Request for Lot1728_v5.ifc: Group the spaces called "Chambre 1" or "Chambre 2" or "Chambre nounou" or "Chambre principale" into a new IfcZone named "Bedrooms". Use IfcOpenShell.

First a look at what the model holds.

```python
import ifcopenshell

model = ifcopenshell.open("Lot1728_v5.ifc")
print(model.schema)
seen = {}
for space in model.by_type("IfcSpace"):
    seen[space.LongName] = seen.get(space.LongName, 0) + 1
for name, count in sorted(seen.items(), key=str):
    print(count, "x", name)
print("zones:", [z.Name for z in model.by_type("IfcZone")][:20])
```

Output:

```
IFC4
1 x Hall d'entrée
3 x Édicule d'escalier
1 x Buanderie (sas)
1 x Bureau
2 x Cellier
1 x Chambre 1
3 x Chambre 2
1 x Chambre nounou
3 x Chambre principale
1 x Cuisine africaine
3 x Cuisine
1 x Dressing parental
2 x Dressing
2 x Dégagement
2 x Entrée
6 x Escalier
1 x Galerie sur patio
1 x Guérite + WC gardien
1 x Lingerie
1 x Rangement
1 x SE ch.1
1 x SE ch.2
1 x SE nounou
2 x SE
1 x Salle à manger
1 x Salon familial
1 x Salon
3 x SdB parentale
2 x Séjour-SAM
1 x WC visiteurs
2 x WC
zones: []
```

```python
import ifcopenshell
import ifcopenshell.api.group
import ifcopenshell.api.root

model = ifcopenshell.open("Lot1728_v5.ifc")

names = {"Chambre 1", "Chambre 2", "Chambre nounou", "Chambre principale"}
spaces = [s for s in model.by_type("IfcSpace") if s.LongName in names]

zone = ifcopenshell.api.root.create_entity(model, ifc_class="IfcZone", name="Bedrooms")
ifcopenshell.api.group.assign_group(model, products=spaces, group=zone)
print(len(spaces), "spaces in", zone.Name)

model.write("Lot1728_v5-out.ifc")
```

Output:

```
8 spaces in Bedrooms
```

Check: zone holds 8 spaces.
